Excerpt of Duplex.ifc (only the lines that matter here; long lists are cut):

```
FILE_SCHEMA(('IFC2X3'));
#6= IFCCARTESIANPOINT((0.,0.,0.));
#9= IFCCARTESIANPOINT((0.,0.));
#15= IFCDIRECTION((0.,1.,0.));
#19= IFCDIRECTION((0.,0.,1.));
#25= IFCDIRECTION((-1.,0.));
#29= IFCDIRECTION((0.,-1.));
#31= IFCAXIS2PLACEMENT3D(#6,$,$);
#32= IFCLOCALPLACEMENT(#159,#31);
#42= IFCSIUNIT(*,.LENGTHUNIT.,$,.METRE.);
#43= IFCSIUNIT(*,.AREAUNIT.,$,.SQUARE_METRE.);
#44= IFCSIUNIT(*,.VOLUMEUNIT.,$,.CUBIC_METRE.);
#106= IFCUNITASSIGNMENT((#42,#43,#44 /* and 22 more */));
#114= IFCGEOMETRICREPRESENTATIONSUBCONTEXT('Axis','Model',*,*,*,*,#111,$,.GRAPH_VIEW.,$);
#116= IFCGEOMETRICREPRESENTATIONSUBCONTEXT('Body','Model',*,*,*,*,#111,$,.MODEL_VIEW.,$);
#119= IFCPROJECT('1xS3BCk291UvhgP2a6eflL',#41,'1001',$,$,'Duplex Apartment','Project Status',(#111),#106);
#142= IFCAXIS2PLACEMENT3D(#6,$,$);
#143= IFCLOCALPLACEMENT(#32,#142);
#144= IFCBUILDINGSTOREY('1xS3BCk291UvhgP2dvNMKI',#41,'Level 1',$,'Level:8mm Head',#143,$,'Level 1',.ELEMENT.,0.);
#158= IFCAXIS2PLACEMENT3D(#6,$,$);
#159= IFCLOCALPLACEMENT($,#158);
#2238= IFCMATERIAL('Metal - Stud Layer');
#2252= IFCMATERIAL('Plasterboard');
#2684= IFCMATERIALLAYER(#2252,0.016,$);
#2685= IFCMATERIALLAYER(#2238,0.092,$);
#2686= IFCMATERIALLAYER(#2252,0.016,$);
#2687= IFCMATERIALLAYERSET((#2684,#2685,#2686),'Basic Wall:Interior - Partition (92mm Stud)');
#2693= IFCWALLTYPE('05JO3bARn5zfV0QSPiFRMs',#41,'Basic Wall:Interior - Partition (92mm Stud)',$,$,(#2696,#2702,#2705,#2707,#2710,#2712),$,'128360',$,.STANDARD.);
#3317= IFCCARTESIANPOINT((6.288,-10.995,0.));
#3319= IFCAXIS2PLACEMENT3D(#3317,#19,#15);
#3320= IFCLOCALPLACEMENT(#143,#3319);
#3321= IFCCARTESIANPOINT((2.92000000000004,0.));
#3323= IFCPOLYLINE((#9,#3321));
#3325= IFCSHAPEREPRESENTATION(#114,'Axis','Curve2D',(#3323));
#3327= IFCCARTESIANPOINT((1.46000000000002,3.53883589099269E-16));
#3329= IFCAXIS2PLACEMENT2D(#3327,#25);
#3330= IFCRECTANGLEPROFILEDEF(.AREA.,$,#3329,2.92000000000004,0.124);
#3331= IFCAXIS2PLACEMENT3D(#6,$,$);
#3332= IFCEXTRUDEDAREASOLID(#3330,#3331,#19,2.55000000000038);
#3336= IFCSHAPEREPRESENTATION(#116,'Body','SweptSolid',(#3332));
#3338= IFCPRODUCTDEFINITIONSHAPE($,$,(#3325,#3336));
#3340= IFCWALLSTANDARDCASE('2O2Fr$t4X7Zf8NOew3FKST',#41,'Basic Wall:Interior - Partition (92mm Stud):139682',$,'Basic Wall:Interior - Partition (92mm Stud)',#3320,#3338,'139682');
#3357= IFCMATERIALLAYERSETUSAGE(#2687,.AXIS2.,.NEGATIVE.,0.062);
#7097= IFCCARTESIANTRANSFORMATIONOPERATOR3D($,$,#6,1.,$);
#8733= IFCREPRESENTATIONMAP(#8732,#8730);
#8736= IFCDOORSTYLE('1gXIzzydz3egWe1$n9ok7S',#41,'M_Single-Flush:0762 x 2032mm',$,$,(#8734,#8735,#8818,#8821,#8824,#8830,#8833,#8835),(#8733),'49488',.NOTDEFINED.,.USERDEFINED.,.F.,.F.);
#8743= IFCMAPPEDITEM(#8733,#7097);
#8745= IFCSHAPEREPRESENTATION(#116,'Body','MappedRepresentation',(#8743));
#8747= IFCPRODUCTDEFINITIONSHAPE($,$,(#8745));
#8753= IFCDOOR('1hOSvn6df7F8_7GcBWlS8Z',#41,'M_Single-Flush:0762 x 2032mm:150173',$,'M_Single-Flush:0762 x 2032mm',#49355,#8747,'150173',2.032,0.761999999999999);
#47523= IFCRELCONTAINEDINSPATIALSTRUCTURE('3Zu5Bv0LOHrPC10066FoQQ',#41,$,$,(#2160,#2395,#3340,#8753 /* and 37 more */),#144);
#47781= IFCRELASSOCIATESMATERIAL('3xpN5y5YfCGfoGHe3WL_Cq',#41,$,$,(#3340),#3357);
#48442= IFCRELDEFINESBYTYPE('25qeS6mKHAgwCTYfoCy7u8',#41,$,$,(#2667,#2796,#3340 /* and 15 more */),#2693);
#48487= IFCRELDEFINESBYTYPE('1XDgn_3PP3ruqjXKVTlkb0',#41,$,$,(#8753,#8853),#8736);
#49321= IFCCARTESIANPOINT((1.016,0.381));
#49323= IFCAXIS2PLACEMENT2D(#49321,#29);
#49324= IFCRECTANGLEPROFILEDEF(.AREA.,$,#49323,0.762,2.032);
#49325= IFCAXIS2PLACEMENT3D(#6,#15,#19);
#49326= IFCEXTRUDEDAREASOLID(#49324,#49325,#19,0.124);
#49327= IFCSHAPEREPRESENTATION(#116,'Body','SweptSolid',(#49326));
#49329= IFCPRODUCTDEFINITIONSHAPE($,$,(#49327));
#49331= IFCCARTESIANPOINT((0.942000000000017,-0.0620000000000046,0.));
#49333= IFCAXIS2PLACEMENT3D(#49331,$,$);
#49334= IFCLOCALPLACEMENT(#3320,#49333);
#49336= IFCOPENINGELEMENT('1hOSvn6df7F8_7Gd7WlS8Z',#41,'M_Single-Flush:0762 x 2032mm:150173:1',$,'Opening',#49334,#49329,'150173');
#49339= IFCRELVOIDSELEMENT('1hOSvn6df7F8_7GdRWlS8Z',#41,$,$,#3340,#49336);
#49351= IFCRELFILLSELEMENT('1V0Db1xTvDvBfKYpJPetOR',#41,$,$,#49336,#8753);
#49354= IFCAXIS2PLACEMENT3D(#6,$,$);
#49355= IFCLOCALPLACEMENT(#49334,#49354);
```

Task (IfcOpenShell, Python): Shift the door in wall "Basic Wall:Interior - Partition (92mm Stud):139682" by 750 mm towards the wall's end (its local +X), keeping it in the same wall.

```python
import ifcopenshell
import ifcopenshell.api.geometry
import ifcopenshell.util.placement
import ifcopenshell.util.unit

model = ifcopenshell.open("Duplex.ifc")
unit_scale = ifcopenshell.util.unit.calculate_unit_scale(model)

door = model.by_guid("1hOSvn6df7F8_7GcBWlS8Z")
opening = door.FillsVoids[0].RelatingOpeningElement
wall = opening.VoidsElements[0].RelatingBuildingElement

wall_matrix = ifcopenshell.util.placement.get_local_placement(wall.ObjectPlacement)
shift = wall_matrix[:3, 0] * 0.75 / unit_scale
before = ifcopenshell.util.placement.get_local_placement(door.ObjectPlacement)[:3, 3].copy()

# The door is placed relative to its opening, so it follows when the opening moves.
matrix = ifcopenshell.util.placement.get_local_placement(opening.ObjectPlacement)
matrix[:3, 3] += shift
ifcopenshell.api.geometry.edit_object_placement(
    model, product=opening, matrix=matrix, is_si=False, should_transform_children=True
)

after = ifcopenshell.util.placement.get_local_placement(door.ObjectPlacement)[:3, 3]
print("door moved by", (after - before).round(3) + 0.0)

model.write("Duplex_edited.ifc")
```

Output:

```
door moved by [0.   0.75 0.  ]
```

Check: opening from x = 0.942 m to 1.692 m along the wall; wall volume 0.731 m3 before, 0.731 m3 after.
